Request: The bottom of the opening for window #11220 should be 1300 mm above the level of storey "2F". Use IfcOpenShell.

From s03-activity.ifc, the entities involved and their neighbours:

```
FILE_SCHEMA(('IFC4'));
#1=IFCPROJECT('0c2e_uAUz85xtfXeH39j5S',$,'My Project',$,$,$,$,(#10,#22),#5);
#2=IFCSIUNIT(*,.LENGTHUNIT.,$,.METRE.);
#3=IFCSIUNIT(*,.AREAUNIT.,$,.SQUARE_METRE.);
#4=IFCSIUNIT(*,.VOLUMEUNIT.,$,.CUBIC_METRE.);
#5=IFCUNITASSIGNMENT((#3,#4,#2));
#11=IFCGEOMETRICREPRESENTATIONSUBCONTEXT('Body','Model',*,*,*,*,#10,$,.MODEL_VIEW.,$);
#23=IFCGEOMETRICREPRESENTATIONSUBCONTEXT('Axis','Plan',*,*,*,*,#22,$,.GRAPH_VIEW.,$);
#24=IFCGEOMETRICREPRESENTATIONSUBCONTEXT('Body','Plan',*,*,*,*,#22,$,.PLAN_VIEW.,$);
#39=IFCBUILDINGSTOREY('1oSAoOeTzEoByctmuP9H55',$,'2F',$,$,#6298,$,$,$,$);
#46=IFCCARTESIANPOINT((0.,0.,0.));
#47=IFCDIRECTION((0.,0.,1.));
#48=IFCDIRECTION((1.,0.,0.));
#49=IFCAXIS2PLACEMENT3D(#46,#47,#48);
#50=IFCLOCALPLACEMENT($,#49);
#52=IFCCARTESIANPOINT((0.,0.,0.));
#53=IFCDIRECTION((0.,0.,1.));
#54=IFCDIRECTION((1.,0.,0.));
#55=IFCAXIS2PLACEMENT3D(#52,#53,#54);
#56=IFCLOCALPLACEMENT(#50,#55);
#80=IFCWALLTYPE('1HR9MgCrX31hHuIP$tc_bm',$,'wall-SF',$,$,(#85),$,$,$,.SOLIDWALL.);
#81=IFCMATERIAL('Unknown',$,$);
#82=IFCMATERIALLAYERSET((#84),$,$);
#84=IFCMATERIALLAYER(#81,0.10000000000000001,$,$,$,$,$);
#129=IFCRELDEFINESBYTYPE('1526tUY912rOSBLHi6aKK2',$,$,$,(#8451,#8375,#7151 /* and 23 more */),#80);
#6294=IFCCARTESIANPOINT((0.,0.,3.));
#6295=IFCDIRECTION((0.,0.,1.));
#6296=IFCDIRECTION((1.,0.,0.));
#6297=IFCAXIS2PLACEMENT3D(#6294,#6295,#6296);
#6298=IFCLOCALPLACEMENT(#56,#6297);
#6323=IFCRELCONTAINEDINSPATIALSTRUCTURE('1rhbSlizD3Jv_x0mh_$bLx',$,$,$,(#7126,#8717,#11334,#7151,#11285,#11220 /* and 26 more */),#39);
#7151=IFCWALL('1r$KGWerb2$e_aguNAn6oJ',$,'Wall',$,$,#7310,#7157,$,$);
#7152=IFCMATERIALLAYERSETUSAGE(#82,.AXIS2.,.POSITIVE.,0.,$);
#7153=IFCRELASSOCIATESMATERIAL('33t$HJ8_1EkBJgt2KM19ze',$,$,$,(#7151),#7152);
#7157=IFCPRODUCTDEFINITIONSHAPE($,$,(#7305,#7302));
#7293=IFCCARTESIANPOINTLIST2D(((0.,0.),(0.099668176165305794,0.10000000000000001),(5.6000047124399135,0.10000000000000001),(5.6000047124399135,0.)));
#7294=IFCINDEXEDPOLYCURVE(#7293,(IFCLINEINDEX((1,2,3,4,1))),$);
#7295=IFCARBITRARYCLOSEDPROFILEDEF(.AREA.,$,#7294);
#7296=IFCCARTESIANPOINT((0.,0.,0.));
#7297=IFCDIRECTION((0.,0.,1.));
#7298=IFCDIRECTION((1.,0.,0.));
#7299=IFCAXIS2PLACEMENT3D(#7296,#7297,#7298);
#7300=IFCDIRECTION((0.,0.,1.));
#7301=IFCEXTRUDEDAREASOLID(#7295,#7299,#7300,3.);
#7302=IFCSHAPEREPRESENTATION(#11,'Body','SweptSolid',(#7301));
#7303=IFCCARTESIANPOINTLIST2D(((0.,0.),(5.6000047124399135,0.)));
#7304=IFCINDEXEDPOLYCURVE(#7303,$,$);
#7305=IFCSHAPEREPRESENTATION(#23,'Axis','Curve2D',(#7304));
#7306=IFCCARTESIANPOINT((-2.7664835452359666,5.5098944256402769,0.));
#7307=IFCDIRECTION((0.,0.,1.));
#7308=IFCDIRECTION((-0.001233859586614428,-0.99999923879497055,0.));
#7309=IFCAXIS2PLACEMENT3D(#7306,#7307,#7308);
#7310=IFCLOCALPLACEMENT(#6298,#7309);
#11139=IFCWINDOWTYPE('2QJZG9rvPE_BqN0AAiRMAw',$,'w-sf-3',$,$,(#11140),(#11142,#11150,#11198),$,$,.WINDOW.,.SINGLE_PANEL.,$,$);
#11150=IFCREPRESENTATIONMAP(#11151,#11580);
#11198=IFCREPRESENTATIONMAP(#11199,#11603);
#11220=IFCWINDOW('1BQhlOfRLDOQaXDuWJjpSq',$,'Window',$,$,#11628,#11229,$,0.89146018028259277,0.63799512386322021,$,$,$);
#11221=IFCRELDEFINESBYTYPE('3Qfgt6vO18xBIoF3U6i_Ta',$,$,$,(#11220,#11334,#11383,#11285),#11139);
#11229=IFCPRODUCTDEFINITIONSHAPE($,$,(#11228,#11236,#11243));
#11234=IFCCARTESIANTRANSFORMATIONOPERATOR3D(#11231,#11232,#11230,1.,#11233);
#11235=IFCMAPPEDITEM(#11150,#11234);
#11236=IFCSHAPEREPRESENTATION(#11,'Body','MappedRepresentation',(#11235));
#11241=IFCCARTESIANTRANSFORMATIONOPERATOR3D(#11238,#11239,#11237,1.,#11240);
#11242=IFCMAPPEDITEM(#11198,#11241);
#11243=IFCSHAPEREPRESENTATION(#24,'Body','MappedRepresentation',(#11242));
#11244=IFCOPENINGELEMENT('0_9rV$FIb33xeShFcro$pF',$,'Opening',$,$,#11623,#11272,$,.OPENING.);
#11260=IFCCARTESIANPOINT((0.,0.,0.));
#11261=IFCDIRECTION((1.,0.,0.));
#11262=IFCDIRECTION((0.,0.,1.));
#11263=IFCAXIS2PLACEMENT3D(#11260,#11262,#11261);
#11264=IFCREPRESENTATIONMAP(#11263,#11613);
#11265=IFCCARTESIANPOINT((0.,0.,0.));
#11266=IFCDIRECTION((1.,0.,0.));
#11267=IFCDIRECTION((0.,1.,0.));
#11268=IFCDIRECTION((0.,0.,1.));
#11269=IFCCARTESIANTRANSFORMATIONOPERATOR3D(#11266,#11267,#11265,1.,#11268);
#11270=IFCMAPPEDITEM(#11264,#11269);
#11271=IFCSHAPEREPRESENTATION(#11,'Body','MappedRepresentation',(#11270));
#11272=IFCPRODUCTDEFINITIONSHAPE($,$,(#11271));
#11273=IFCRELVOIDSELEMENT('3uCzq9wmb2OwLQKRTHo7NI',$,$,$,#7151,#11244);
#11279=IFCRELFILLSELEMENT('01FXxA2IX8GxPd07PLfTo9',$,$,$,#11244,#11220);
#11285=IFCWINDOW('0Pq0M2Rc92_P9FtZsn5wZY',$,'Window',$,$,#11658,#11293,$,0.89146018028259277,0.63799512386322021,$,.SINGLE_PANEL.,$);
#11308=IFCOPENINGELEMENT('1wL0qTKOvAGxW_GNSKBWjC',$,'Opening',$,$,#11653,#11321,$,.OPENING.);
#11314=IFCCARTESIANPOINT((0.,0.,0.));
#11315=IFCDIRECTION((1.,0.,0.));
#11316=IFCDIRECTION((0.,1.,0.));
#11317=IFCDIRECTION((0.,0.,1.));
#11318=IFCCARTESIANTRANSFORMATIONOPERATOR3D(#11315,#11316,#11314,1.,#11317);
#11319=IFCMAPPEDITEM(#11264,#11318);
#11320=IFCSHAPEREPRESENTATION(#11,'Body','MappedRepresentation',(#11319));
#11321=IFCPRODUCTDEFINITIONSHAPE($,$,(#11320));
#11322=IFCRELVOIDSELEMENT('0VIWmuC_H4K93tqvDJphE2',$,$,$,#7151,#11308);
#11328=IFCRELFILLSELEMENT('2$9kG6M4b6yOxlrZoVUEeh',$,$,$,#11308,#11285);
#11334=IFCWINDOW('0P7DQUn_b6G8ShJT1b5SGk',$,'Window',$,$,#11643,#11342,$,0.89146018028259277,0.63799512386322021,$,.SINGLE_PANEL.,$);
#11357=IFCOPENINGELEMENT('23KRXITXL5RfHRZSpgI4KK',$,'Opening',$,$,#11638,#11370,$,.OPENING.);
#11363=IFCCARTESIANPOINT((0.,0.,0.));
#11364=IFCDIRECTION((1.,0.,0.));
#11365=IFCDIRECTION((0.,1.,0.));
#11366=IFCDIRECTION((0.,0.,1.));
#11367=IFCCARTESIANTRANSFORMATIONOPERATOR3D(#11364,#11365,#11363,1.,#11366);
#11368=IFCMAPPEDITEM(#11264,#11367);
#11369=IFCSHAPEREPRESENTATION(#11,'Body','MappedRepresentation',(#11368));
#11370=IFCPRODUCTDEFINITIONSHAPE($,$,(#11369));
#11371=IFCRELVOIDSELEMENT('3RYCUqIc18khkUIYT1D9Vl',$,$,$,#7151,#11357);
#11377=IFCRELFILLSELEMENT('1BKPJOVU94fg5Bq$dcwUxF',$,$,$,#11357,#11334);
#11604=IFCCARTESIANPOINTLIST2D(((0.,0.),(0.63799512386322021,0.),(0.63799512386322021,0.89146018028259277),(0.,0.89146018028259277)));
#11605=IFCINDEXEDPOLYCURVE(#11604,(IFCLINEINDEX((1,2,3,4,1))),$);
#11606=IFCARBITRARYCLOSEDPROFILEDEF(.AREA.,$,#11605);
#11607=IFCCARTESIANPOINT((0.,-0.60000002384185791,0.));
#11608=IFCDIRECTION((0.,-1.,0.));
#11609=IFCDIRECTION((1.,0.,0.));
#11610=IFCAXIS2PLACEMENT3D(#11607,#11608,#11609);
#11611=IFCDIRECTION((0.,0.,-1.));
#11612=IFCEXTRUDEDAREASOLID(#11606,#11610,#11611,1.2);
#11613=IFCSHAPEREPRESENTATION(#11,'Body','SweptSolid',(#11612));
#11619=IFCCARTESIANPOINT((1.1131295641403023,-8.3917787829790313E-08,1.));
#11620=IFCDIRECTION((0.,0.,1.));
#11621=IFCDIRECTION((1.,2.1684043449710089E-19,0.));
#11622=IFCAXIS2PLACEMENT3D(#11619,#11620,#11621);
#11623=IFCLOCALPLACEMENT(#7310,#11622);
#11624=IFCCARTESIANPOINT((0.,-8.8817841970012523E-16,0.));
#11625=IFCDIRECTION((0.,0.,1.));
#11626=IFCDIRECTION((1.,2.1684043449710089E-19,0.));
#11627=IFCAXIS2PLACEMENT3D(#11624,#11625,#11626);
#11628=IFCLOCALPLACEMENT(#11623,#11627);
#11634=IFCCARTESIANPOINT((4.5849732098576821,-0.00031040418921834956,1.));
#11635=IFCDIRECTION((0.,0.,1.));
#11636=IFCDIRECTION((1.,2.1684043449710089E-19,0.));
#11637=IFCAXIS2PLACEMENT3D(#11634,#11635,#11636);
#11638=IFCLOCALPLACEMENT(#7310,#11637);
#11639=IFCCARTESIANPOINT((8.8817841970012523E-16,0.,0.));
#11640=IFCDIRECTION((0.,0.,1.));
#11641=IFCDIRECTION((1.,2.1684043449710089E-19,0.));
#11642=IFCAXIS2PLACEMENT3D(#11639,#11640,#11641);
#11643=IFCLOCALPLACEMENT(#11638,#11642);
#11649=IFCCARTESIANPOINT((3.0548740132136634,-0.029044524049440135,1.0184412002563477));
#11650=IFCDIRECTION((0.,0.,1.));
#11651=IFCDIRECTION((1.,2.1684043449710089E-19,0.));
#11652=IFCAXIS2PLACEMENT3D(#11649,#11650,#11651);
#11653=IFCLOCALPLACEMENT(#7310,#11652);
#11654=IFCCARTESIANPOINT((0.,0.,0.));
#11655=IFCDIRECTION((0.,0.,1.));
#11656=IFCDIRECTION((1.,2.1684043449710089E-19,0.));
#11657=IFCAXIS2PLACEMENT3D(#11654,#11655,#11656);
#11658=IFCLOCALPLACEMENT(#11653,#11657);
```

```python
import numpy as np
import ifcopenshell
import ifcopenshell.api.geometry
import ifcopenshell.geom
import ifcopenshell.util.element
import ifcopenshell.util.placement
import ifcopenshell.util.shape
import ifcopenshell.util.unit

model = ifcopenshell.open("s03-activity.ifc")
unit_scale = ifcopenshell.util.unit.calculate_unit_scale(model)

window = model.by_guid("1BQhlOfRLDOQaXDuWJjpSq")
opening = window.FillsVoids[0].RelatingOpeningElement
storey = ifcopenshell.util.element.get_container(window, ifc_class="IfcBuildingStorey")
level = ifcopenshell.util.placement.get_local_placement(storey.ObjectPlacement)[2, 3]

# The opening's origin need not be at the sill, so measure its lowest point.
shape = ifcopenshell.geom.create_shape(ifcopenshell.geom.settings(), opening)
bottom = ifcopenshell.util.shape.get_shape_bottom_elevation(shape, shape.geometry) / unit_scale
dz = level + 1.3 - bottom

shift = np.array([0.0, 0.0, dz])
# The window is placed relative to its opening, so it follows when the opening moves.
matrix = ifcopenshell.util.placement.get_local_placement(opening.ObjectPlacement)
matrix[:3, 3] += shift
ifcopenshell.api.geometry.edit_object_placement(
    model, product=opening, matrix=matrix, is_si=False, should_transform_children=True
)

print(f"moved by {dz * unit_scale:+.3f} m")

model.write("s03-activity_rev.ifc")
```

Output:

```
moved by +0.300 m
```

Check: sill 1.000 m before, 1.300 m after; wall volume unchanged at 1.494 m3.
